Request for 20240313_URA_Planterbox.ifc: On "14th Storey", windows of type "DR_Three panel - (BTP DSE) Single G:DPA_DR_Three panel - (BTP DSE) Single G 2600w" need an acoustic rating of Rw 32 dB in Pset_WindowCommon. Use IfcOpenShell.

First a look at what the model holds.

```python
import ifcopenshell
import ifcopenshell.util.element

model = ifcopenshell.open("20240313_URA_Planterbox.ifc")
print(model.schema)
storey = next(s for s in model.by_type("IfcBuildingStorey") if s.Name == "14th Storey")
windows = [e for e in ifcopenshell.util.element.get_decomposition(storey) if e.is_a("IfcWindow")]
seen = {}
for e in windows:
    element_type = ifcopenshell.util.element.get_type(e)
    key = (element_type.Name if element_type != e and element_type else None, ifcopenshell.util.element.get_pset(e, "Pset_WindowCommon", "AcousticRating"))
    seen[key] = seen.get(key, 0) + 1
for (name, value), count in sorted(seen.items(), key=str):
    print(count, "x", name, "|", value)
```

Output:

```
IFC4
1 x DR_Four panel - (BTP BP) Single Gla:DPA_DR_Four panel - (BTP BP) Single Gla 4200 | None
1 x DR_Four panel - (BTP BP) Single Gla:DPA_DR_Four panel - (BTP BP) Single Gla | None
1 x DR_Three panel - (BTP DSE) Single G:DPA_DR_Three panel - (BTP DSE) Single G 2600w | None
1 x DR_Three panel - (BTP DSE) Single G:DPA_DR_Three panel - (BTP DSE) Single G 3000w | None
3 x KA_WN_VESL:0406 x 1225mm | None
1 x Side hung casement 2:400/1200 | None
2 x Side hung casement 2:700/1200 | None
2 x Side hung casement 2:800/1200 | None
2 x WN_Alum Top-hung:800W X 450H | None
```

```python
import ifcopenshell
import ifcopenshell.api.pset
import ifcopenshell.util.element

model = ifcopenshell.open("20240313_URA_Planterbox.ifc")

storey = next(s for s in model.by_type("IfcBuildingStorey") if s.Name == "14th Storey")
windows = [e for e in ifcopenshell.util.element.get_decomposition(storey) if e.is_a("IfcWindow")]

count = 0
for e in windows:
    element_type = ifcopenshell.util.element.get_type(e)
    if element_type in (None, e) or element_type.Name != "DR_Three panel - (BTP DSE) Single G:DPA_DR_Three panel - (BTP DSE) Single G 2600w":
        continue
    # add_pset returns the element's existing set when there is one.
    pset = ifcopenshell.api.pset.add_pset(model, product=e, name="Pset_WindowCommon")
    ifcopenshell.api.pset.edit_pset(model, pset=pset, properties={"AcousticRating": "Rw 32 dB"})
    count += 1

print(count, "windows updated")

model.write("20240313_URA_Planterbox-out.ifc")
```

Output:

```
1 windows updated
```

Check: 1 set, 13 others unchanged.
